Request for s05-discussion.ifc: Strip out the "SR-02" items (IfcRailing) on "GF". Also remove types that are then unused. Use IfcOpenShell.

First a look at what the model holds.

```python
import ifcopenshell
import ifcopenshell.util.element

model = ifcopenshell.open("s05-discussion.ifc")
print(model.schema)
storey = next(s for s in model.by_type("IfcBuildingStorey") if s.Name == "GF")
railings = [e for e in ifcopenshell.util.element.get_decomposition(storey) if e.is_a("IfcRailing")]
seen = {}
for e in railings:
    element_type = ifcopenshell.util.element.get_type(e)
    name = element_type.Name if element_type not in (None, e) else None
    seen[name] = seen.get(name, 0) + 1
for name, count in sorted(seen.items(), key=str):
    print(count, "x", name)
```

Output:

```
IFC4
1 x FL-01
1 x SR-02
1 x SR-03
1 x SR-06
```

```python
import ifcopenshell
import ifcopenshell.api.root
import ifcopenshell.util.element

model = ifcopenshell.open("s05-discussion.ifc")

storey = next(s for s in model.by_type("IfcBuildingStorey") if s.Name == "GF")
railings = [e for e in ifcopenshell.util.element.get_decomposition(storey) if e.is_a("IfcRailing")]
targets = [e for e in railings if (t := ifcopenshell.util.element.get_type(e)) not in (None, e) and t.Name == "SR-02"]
types = {ifcopenshell.util.element.get_type(e) for e in targets} - {None, *targets}

for e in targets:
    ifcopenshell.api.root.remove_product(model, product=e)
print(len(targets), "removed")

unused = [t for t in types if not ifcopenshell.util.element.get_types(t)]
for t in unused:
    ifcopenshell.api.root.remove_product(model, product=t)
print(len(unused), "unused types removed")

model.write("s05-discussion_updated.ifc")
```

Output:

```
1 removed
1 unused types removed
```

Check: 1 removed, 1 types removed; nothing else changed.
